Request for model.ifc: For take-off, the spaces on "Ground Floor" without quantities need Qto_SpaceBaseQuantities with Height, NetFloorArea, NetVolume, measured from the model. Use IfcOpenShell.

First a look at what the model holds.

```python
import ifcopenshell
import ifcopenshell.util.element
import ifcopenshell.util.unit

model = ifcopenshell.open("model.ifc")
print(model.schema)
for unit_type in ("LENGTHUNIT", "AREAUNIT", "VOLUMEUNIT"):
    print(unit_type, ifcopenshell.util.unit.calculate_unit_scale(model, unit_type))
storey = next(s for s in model.by_type("IfcBuildingStorey") if s.Name == "Ground Floor")
spaces = [e for e in ifcopenshell.util.element.get_decomposition(storey) if e.is_a("IfcSpace")]
for e in sorted(spaces, key=lambda e: e.id()):
    print(e.id(), e.is_a(), e.Name, list(ifcopenshell.util.element.get_psets(e, qtos_only=True)), sep=" | ")
```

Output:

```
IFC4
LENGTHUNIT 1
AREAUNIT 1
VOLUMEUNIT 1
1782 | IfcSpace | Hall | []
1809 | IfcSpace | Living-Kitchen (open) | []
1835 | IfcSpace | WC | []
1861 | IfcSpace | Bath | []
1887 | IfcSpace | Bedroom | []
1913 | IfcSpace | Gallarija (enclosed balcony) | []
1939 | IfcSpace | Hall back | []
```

```python
import ifcopenshell
import ifcopenshell.api.pset
import ifcopenshell.geom
import ifcopenshell.util.element
import ifcopenshell.util.shape
import ifcopenshell.util.unit

model = ifcopenshell.open("model.ifc")
unit_scale = ifcopenshell.util.unit.calculate_unit_scale(model)
area_scale = ifcopenshell.util.unit.calculate_unit_scale(model, "AREAUNIT")
volume_scale = ifcopenshell.util.unit.calculate_unit_scale(model, "VOLUMEUNIT")
settings = ifcopenshell.geom.settings()

storey = next(s for s in model.by_type("IfcBuildingStorey") if s.Name == "Ground Floor")
spaces = [e for e in ifcopenshell.util.element.get_decomposition(storey) if e.is_a("IfcSpace")]

for e in sorted(spaces, key=lambda e: e.id()):
    if ifcopenshell.util.element.get_psets(e, qtos_only=True, should_inherit=False):
        continue
    # Geometry comes back in metres, in the element's own axes.
    shape = ifcopenshell.geom.create_shape(settings, e)
    values = {
        "Height": ifcopenshell.util.shape.get_z(shape.geometry) / unit_scale,
        "NetFloorArea": ifcopenshell.util.shape.get_footprint_area(shape.geometry) / area_scale,
        "NetVolume": ifcopenshell.util.shape.get_volume(shape.geometry) / volume_scale,
    }
    qto = ifcopenshell.api.pset.add_qto(model, product=e, name="Qto_SpaceBaseQuantities")
    ifcopenshell.api.pset.edit_qto(model, qto=qto, properties=values)
    print(e.id(), {k: round(v, 3) for k, v in values.items()})

model.write("model-out.ifc")
```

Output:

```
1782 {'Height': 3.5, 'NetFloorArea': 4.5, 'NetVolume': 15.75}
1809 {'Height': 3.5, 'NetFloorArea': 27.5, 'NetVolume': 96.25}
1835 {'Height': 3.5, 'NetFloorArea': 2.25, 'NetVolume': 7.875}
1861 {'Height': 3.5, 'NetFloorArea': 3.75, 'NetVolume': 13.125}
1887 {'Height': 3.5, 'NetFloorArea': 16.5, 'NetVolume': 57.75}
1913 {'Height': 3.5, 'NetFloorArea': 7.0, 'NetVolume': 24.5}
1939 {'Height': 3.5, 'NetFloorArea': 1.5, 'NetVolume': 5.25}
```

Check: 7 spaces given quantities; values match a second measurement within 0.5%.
